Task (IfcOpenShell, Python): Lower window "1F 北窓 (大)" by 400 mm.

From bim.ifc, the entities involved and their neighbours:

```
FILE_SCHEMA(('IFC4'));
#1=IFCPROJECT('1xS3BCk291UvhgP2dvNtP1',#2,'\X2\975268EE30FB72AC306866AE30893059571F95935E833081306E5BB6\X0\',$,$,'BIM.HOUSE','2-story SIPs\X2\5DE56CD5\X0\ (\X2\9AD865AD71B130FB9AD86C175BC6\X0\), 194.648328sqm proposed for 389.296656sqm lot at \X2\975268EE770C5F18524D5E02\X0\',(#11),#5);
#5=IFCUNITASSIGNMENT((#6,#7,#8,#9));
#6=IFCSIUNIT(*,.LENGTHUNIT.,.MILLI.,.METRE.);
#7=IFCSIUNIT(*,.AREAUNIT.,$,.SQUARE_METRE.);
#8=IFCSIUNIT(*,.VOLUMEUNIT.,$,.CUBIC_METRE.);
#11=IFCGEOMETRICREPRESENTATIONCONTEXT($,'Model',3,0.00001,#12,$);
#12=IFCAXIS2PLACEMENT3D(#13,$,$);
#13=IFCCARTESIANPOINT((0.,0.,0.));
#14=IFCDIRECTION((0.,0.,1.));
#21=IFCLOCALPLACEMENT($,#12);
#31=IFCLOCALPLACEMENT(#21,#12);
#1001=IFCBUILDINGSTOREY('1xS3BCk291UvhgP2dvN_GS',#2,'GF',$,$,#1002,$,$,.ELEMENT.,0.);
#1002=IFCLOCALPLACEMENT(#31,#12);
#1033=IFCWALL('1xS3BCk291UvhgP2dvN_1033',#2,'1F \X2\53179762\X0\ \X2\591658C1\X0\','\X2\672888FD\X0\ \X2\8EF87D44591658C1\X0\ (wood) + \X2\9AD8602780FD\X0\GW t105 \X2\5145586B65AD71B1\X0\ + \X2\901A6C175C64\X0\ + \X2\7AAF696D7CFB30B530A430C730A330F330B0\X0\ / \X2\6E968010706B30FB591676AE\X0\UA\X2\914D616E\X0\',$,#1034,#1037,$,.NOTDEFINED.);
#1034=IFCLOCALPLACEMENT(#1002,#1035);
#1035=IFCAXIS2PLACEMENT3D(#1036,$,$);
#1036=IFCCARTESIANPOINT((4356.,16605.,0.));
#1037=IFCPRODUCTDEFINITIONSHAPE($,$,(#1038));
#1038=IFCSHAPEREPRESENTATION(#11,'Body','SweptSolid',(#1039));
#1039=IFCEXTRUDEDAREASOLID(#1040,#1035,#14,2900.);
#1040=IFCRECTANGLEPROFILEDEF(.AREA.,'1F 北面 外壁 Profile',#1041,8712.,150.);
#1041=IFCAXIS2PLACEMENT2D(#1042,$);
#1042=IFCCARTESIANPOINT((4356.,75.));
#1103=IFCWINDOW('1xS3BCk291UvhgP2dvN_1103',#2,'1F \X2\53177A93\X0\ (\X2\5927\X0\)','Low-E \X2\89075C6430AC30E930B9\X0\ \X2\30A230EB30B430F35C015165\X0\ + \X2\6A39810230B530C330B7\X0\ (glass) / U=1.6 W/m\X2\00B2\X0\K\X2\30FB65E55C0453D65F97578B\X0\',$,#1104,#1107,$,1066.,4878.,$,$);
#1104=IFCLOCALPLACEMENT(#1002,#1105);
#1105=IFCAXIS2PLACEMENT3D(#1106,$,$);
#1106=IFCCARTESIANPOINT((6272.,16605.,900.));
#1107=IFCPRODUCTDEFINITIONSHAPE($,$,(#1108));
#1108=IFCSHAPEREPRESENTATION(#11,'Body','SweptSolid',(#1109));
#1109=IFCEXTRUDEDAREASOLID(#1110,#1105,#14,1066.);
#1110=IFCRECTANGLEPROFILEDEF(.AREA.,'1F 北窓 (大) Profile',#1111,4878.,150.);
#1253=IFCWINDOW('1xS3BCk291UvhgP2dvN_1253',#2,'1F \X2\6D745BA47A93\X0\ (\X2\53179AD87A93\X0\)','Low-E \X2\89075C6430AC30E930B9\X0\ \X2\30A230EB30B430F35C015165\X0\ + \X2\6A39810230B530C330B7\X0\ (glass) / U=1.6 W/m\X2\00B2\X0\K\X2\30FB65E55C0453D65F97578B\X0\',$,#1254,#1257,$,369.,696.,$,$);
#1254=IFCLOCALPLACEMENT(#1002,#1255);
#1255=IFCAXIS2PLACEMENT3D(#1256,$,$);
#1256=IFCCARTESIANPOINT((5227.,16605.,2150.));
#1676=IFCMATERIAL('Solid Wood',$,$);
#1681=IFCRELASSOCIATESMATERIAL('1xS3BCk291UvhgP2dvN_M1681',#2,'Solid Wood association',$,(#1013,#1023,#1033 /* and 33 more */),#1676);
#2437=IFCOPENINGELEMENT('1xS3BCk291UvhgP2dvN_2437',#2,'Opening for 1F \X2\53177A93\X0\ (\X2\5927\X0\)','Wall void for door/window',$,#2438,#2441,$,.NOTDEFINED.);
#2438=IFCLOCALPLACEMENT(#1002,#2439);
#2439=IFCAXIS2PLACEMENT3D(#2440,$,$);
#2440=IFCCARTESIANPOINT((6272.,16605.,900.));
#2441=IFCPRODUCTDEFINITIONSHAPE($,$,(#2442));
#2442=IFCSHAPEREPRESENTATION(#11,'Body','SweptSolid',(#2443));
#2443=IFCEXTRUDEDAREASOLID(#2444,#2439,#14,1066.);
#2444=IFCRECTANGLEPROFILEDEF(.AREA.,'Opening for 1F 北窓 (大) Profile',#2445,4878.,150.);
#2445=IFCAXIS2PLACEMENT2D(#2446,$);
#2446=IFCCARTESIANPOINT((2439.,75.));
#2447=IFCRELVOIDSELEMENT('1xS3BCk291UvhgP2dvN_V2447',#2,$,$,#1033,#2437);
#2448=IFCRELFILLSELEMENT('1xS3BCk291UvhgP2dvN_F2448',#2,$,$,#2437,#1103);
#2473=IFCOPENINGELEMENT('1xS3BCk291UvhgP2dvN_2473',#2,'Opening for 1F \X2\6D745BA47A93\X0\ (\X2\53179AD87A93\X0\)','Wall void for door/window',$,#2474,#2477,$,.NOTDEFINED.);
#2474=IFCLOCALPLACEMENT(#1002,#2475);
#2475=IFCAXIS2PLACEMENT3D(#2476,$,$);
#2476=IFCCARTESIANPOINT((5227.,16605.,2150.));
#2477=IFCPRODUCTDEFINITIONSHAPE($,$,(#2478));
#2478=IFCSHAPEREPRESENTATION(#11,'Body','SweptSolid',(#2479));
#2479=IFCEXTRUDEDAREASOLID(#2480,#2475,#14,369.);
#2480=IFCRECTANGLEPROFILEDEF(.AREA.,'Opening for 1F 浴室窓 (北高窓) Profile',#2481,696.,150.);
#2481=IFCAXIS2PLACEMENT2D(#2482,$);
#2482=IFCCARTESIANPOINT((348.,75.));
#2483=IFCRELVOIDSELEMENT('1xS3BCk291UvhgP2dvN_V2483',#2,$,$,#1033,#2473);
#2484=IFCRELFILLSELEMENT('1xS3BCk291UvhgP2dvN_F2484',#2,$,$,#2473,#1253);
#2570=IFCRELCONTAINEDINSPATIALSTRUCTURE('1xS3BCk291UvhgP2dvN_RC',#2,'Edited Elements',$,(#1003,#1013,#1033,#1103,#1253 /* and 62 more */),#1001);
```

```python
import numpy as np
import ifcopenshell
import ifcopenshell.api.geometry
import ifcopenshell.util.placement
import ifcopenshell.util.unit

model = ifcopenshell.open("bim.ifc")
unit_scale = ifcopenshell.util.unit.calculate_unit_scale(model)

window = model.by_guid("1xS3BCk291UvhgP2dvN_1103")
opening = window.FillsVoids[0].RelatingOpeningElement
dz = -400.0

shift = np.array([0.0, 0.0, dz])
# The window is not placed relative to its opening, so move both.
for product in (opening, window):
    matrix = ifcopenshell.util.placement.get_local_placement(product.ObjectPlacement)
    matrix[:3, 3] += shift
    ifcopenshell.api.geometry.edit_object_placement(model, product=product, matrix=matrix, is_si=False)

print(f"moved by {dz * unit_scale:+.3f} m")

model.write("bim_updated.ifc")
```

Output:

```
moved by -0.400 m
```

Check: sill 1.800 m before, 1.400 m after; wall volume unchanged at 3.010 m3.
